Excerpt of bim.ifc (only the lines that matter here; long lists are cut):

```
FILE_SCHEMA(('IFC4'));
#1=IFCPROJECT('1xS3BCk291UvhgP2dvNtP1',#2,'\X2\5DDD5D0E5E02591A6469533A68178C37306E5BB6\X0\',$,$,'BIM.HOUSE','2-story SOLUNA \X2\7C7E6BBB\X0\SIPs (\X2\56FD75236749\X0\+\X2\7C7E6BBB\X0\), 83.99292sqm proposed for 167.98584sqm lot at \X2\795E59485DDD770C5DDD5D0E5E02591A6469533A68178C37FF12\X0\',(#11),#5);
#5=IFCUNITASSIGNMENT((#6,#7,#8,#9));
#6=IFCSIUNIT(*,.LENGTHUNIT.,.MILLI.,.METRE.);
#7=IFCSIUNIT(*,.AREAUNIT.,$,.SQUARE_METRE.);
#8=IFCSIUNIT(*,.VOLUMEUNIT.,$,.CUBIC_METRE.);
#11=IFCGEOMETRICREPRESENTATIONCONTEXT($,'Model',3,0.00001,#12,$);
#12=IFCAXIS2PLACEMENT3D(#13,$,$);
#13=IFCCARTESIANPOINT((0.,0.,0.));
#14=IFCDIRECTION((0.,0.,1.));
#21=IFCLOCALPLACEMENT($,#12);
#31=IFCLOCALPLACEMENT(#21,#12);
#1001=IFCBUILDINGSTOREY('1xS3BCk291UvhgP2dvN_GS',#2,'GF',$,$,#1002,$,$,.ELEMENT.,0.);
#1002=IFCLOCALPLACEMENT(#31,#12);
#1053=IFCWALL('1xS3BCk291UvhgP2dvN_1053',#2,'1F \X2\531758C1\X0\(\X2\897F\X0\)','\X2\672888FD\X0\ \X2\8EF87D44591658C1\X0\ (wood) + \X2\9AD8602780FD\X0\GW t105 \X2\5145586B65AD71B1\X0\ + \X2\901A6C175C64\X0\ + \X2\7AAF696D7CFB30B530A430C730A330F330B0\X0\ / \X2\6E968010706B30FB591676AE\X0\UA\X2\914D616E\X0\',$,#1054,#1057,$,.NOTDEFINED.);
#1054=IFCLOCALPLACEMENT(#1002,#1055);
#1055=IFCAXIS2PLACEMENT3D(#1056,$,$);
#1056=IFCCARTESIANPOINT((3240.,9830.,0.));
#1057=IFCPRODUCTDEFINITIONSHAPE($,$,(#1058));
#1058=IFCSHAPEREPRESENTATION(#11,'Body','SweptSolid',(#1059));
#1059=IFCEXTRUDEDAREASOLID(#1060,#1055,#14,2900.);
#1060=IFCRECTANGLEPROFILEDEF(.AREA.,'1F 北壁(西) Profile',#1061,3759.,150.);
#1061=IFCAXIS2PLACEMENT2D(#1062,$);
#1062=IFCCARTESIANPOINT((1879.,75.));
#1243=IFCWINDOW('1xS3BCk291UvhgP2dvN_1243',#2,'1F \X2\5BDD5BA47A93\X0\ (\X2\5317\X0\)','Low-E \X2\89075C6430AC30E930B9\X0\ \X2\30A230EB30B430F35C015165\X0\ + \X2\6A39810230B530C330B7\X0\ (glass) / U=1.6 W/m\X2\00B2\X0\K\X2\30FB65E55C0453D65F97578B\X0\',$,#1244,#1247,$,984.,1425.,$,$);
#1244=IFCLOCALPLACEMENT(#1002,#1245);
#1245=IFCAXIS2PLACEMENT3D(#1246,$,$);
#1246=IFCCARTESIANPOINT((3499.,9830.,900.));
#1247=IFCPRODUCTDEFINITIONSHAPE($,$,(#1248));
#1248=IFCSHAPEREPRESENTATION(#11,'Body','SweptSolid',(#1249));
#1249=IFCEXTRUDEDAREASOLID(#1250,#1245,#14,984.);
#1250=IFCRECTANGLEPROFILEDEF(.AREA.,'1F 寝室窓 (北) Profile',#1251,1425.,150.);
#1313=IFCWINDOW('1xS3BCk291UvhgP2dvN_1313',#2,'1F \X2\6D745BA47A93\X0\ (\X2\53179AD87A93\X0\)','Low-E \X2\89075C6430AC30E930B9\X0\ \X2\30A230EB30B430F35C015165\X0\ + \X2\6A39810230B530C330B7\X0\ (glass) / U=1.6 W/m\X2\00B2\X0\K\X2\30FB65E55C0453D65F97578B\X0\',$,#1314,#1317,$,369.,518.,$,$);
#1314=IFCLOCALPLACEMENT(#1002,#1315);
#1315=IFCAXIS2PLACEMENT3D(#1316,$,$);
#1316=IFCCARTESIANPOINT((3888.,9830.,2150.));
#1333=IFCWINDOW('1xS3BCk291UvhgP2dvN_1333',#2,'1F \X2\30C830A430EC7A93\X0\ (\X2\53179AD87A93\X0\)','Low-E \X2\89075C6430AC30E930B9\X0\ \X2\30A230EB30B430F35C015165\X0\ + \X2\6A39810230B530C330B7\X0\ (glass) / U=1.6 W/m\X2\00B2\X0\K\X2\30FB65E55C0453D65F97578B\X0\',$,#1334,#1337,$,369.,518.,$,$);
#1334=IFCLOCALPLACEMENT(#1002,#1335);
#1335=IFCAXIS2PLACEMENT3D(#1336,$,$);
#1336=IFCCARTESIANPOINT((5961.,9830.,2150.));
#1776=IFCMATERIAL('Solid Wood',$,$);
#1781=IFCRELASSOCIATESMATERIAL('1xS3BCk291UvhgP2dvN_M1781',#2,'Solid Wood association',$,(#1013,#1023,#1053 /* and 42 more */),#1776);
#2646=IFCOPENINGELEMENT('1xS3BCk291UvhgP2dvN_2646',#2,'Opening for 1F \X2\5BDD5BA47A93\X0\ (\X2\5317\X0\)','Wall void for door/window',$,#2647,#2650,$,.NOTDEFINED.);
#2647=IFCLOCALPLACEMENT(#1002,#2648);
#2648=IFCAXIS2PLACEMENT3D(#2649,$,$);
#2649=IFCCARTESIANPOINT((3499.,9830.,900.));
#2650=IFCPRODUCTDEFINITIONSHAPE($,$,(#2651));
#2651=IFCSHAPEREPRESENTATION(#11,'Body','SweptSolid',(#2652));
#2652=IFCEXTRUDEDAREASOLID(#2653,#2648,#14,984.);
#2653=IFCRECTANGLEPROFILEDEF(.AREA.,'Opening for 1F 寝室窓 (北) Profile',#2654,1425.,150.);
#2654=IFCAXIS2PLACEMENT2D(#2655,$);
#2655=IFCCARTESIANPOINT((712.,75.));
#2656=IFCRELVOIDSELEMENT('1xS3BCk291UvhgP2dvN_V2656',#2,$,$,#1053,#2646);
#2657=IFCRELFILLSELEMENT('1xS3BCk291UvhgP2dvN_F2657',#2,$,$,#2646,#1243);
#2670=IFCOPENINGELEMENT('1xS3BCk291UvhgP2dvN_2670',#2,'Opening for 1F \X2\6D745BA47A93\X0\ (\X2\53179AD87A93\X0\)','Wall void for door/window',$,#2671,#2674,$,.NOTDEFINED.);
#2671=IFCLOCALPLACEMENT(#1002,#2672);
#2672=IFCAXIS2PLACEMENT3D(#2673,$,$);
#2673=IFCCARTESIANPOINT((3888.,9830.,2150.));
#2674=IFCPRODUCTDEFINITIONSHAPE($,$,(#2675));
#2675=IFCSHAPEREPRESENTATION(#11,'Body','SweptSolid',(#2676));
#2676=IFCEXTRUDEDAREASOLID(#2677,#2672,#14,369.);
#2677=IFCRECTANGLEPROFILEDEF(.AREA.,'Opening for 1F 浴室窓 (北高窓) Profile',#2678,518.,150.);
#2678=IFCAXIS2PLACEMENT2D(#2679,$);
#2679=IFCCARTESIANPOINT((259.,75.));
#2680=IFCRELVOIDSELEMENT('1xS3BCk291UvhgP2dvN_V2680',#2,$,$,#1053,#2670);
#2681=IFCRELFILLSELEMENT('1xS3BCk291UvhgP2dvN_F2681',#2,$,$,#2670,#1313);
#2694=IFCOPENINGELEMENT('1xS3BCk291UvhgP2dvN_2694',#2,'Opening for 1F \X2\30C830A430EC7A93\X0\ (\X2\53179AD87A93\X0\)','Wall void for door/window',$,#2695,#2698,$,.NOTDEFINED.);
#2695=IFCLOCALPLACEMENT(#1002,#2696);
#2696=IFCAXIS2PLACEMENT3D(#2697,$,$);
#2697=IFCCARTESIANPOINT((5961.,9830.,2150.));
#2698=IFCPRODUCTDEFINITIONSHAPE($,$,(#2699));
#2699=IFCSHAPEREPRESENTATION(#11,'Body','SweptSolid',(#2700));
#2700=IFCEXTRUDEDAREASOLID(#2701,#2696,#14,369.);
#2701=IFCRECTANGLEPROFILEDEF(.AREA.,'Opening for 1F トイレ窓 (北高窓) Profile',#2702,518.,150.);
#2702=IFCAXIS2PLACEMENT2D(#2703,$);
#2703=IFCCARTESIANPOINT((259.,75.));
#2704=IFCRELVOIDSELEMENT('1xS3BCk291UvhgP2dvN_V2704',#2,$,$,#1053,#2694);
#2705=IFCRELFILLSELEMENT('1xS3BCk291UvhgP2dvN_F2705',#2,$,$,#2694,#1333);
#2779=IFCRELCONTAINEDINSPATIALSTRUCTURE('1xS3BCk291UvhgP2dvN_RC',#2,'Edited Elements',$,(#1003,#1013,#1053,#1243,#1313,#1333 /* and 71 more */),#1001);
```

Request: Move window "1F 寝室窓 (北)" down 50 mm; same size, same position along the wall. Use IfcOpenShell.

```python
import numpy as np
import ifcopenshell
import ifcopenshell.api.geometry
import ifcopenshell.util.placement
import ifcopenshell.util.unit

model = ifcopenshell.open("bim.ifc")
unit_scale = ifcopenshell.util.unit.calculate_unit_scale(model)

window = model.by_id(1243)
opening = window.FillsVoids[0].RelatingOpeningElement
dz = -50.0

shift = np.array([0.0, 0.0, dz])
# The window is not placed relative to its opening, so move both.
for product in (opening, window):
    matrix = ifcopenshell.util.placement.get_local_placement(product.ObjectPlacement)
    matrix[:3, 3] += shift
    ifcopenshell.api.geometry.edit_object_placement(model, product=product, matrix=matrix, is_si=False)

print(f"moved by {dz * unit_scale:+.3f} m")

model.write("bim_edited.ifc")
```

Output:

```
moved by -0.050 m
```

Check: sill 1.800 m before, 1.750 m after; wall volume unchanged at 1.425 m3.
